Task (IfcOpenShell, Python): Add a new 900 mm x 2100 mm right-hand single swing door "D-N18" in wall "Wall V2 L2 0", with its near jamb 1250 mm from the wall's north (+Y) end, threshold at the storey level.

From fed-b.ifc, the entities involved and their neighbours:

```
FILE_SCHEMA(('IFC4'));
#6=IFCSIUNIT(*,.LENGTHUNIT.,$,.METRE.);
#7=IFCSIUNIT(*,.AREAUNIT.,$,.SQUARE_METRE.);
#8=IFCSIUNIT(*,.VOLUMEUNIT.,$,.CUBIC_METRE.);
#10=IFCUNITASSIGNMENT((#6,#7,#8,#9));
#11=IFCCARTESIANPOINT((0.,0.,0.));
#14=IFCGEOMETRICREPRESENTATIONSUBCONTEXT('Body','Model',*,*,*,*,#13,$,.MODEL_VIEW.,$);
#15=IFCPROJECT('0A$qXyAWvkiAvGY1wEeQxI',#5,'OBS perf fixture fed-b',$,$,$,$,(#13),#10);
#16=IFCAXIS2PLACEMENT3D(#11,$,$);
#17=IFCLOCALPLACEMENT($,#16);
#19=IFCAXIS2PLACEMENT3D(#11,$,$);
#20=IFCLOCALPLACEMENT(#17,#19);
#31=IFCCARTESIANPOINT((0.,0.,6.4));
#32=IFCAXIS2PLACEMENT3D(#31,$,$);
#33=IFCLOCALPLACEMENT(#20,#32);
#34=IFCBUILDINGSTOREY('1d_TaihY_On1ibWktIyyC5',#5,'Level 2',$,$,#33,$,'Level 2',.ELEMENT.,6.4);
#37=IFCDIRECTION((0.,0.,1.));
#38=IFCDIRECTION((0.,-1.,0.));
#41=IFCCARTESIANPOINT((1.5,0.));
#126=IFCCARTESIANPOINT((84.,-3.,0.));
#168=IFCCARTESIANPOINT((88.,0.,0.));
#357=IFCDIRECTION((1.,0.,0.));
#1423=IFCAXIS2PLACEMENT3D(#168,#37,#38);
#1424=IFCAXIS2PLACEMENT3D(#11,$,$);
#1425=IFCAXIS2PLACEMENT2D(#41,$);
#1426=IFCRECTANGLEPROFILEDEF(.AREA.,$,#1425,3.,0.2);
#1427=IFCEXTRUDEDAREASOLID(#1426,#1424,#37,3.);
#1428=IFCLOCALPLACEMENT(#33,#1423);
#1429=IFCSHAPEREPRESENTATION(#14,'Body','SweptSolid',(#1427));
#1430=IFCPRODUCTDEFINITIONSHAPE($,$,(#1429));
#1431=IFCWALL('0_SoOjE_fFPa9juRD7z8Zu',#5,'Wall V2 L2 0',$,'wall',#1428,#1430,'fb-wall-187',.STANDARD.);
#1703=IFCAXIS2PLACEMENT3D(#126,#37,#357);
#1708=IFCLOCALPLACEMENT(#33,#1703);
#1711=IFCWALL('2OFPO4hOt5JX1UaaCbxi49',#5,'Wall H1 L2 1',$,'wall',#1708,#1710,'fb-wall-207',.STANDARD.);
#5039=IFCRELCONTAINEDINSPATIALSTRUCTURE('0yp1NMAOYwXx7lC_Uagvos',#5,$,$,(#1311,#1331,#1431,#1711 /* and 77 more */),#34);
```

```python
import numpy as np
import ifcopenshell
import ifcopenshell.api.feature
import ifcopenshell.api.geometry
import ifcopenshell.api.root
import ifcopenshell.api.spatial
import ifcopenshell.geom
import ifcopenshell.util.element
import ifcopenshell.util.placement
import ifcopenshell.util.representation
import ifcopenshell.util.shape
import ifcopenshell.util.unit

model = ifcopenshell.open("fed-b.ifc")
unit_scale = ifcopenshell.util.unit.calculate_unit_scale(model)
settings = ifcopenshell.geom.settings()


def volume(element):
    """Net volume in cubic metres, openings subtracted."""
    shape = ifcopenshell.geom.create_shape(settings, element)
    return ifcopenshell.util.shape.get_volume(shape.geometry)


wall = model.by_guid("0_SoOjE_fFPa9juRD7z8Zu")
storey = ifcopenshell.util.element.get_container(wall, ifc_class="IfcBuildingStorey")
context = ifcopenshell.util.representation.get_context(model, "Model", "Body", "MODEL_VIEW")
before = volume(wall)

width, height, from_end, sill = 0.9, 2.1, 1.25, 0.0  # metres

# The wall runs along its own X axis, and the end named is its -X end.
wall_shape = ifcopenshell.geom.create_shape(settings, wall)
x, y, z = ifcopenshell.util.shape.get_vertices(wall_shape.geometry).T
start = x.min() + from_end
face, thickness = float(y.min()), float(y.max() - y.min())
wall_matrix = ifcopenshell.util.placement.get_local_placement(wall.ObjectPlacement)
level = ifcopenshell.util.placement.get_local_placement(storey.ObjectPlacement)[2, 3]


def in_wall(x, y):
    """Placement at x, y metres in the wall's axes, at sill height."""
    matrix = wall_matrix.copy()
    matrix[:, 3] = wall_matrix @ np.array([x / unit_scale, y / unit_scale, 0.0, 1.0])
    matrix[2, 3] = level + sill / unit_scale
    return matrix


# Opening: a box that overshoots both wall faces by 50 mm.
opening = ifcopenshell.api.root.create_entity(model, ifc_class="IfcOpeningElement", predefined_type="OPENING")
box = ifcopenshell.api.geometry.add_wall_representation(
    model, context=context, length=width, height=height, thickness=thickness + 0.1
)
ifcopenshell.api.geometry.assign_representation(model, product=opening, representation=box)
ifcopenshell.api.geometry.edit_object_placement(model, product=opening, matrix=in_wall(start, face - 0.05), is_si=False)
ifcopenshell.api.feature.add_feature(model, feature=opening, element=wall)

door = ifcopenshell.api.root.create_entity(model, ifc_class="IfcDoor", name="D-N18", predefined_type="DOOR")
door.OverallWidth, door.OverallHeight = width / unit_scale, height / unit_scale
door.OperationType = "SINGLE_SWING_RIGHT"
body = ifcopenshell.api.geometry.add_door_representation(
    model,
    context=context,
    overall_width=door.OverallWidth,
    overall_height=door.OverallHeight,
    operation_type="SINGLE_SWING_RIGHT",
    lining_properties={"LiningDepth": thickness / unit_scale, "ThresholdDepth": thickness / unit_scale},
)
ifcopenshell.api.geometry.assign_representation(model, product=door, representation=body)
ifcopenshell.api.spatial.assign_container(model, products=[door], relating_structure=storey)
ifcopenshell.api.feature.add_filling(model, opening=opening, element=door)

# The lining spans the wall, so the door starts at the wall face.
ifcopenshell.api.geometry.edit_object_placement(model, product=door, matrix=in_wall(start, face), is_si=False)

after = volume(wall)

print(f"wall volume {before:.3f} -> {after:.3f} m3")

model.write("fed-b_rev.ifc")
```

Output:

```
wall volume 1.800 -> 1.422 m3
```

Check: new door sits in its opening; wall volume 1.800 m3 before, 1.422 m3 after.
